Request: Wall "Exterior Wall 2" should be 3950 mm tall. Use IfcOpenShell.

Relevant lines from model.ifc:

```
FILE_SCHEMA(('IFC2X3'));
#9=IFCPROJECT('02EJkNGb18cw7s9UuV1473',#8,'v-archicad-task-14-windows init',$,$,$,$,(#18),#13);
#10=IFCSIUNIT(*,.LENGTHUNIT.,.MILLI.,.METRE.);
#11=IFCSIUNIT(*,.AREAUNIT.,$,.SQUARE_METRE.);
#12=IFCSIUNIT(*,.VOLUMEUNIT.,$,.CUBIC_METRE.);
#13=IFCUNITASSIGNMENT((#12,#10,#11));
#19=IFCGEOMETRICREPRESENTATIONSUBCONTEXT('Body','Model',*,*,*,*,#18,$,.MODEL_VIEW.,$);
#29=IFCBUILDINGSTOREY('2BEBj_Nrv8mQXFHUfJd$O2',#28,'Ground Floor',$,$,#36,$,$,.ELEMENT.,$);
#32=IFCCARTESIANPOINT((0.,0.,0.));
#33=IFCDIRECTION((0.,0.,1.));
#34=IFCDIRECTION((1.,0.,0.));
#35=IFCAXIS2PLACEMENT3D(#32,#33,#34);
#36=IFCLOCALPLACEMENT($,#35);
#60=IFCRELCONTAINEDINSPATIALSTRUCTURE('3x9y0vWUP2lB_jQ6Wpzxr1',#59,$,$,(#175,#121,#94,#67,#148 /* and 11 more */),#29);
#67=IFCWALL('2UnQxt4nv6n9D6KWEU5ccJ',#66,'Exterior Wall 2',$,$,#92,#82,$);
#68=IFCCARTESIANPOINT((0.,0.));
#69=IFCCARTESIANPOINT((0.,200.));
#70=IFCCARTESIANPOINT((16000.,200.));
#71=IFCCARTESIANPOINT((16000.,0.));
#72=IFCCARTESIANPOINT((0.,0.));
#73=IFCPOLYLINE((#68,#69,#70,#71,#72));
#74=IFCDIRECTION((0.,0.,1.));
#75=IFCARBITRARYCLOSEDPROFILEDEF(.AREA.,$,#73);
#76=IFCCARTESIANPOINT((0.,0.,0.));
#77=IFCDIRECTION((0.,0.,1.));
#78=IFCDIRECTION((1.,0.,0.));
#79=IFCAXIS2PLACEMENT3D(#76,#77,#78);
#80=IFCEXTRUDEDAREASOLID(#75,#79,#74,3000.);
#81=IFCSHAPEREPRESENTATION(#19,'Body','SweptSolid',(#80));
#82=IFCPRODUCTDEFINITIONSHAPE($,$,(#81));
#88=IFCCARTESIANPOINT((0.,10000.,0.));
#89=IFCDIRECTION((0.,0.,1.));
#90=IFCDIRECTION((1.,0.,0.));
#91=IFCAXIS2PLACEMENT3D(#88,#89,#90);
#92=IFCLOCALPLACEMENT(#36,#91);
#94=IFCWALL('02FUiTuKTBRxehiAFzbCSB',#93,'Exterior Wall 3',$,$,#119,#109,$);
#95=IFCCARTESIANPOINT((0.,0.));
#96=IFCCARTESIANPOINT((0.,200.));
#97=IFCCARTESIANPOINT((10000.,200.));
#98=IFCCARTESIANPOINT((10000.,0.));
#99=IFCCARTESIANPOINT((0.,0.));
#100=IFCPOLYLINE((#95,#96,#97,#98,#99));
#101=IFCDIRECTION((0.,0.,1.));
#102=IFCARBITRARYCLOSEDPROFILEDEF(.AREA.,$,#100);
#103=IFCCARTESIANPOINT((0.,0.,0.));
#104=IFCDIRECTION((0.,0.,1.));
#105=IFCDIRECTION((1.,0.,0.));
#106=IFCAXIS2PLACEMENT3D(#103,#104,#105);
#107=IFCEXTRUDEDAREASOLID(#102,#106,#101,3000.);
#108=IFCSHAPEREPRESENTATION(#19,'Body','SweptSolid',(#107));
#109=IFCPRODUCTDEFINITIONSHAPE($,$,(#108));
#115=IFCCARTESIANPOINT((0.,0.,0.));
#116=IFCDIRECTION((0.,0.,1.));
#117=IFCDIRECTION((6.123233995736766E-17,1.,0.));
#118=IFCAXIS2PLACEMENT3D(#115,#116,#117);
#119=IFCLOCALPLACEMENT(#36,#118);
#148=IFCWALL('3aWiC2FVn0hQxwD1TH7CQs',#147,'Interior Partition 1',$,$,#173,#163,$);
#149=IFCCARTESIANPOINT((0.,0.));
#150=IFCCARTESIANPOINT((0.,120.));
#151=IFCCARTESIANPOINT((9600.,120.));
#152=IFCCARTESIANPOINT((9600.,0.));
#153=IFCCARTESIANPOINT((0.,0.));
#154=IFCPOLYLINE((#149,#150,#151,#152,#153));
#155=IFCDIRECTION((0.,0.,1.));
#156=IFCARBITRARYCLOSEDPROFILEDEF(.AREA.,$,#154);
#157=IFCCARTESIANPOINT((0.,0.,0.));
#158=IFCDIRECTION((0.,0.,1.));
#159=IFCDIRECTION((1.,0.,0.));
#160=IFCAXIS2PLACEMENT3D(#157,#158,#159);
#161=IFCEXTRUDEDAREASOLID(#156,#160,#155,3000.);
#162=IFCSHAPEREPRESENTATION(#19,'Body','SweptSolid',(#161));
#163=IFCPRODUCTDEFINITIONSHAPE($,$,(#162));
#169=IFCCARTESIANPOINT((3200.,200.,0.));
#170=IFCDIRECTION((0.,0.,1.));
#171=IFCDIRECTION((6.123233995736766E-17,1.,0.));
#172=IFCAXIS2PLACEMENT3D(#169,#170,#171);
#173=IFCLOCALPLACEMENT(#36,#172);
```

```python
import ifcopenshell
import ifcopenshell.geom
import ifcopenshell.util.representation
import ifcopenshell.util.shape

model = ifcopenshell.open("model.ifc")
settings = ifcopenshell.geom.settings()


def volume(element):
    """Net volume in cubic metres, openings subtracted."""
    shape = ifcopenshell.geom.create_shape(settings, element)
    return ifcopenshell.util.shape.get_volume(shape.geometry)


wall = model.by_guid("2UnQxt4nv6n9D6KWEU5ccJ")
before = volume(wall)

body = ifcopenshell.util.representation.get_representation(wall, "Model", "Body")
solid = body.Items[0]
old_height = solid.Depth
solid.Depth = 3950.0
after = volume(wall)

print(f"height {old_height:g} -> {solid.Depth:g}, volume {before:.3f} -> {after:.3f} m3")

model.write("model_rev.ifc")
```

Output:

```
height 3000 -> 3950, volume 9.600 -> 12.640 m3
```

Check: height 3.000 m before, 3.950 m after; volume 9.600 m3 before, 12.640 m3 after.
